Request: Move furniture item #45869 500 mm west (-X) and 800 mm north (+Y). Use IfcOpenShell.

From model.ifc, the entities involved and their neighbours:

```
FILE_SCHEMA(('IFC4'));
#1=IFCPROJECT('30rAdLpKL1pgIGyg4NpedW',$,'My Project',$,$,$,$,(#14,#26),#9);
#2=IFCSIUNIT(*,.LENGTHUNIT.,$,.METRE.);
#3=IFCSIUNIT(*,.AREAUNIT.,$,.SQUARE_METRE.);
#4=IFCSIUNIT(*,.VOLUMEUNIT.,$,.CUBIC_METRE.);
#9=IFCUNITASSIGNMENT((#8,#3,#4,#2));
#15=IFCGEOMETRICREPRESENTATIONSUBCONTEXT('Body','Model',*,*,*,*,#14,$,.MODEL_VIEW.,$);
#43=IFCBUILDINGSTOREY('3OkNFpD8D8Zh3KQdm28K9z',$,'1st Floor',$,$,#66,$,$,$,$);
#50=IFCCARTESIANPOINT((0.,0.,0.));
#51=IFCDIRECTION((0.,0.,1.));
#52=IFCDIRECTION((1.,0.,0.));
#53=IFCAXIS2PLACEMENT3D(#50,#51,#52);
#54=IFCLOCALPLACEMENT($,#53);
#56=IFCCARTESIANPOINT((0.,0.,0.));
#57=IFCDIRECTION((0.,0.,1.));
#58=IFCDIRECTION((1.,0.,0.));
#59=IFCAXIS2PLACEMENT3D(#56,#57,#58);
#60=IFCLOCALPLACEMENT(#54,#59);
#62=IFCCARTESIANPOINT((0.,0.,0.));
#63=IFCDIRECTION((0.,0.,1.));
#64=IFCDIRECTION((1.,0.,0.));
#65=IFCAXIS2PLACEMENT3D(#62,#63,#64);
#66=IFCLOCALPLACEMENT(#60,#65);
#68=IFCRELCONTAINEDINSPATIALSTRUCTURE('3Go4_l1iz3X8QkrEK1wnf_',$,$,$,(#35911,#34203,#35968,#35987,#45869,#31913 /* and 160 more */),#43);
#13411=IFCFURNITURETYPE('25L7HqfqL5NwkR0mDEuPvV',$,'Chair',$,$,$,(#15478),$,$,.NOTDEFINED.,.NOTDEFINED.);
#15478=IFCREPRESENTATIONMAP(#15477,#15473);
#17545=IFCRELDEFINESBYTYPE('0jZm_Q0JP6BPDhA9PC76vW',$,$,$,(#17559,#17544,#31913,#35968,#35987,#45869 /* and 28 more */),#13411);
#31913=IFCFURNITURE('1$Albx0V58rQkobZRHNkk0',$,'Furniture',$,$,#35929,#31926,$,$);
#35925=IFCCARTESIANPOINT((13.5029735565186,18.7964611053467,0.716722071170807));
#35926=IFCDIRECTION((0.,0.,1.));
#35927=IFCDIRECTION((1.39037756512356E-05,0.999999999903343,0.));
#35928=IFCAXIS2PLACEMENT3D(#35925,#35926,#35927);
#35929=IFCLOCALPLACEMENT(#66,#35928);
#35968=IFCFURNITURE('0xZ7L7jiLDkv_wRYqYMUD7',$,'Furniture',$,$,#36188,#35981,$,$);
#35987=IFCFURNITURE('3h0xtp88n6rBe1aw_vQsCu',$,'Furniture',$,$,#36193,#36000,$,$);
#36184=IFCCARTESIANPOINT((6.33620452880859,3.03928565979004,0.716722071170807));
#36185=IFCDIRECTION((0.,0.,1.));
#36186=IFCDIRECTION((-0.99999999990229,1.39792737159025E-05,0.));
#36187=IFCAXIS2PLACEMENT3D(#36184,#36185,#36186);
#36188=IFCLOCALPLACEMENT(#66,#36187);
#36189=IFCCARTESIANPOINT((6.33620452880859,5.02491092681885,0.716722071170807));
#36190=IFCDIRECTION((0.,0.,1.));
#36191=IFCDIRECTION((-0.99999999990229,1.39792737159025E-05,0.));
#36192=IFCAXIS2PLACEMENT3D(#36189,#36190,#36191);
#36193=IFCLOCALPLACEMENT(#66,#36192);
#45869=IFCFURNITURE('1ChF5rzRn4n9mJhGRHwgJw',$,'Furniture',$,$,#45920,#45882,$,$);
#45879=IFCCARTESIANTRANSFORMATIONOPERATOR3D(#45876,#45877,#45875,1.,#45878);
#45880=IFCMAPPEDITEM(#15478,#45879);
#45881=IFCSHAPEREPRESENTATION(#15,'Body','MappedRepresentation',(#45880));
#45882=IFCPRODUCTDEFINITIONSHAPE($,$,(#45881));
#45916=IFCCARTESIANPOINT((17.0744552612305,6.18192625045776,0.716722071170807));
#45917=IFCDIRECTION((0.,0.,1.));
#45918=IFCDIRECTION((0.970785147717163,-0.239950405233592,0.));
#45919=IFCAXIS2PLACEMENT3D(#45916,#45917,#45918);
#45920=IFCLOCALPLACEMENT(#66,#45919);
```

```python
import ifcopenshell
import ifcopenshell.api.geometry
import ifcopenshell.util.placement
import ifcopenshell.util.unit

model = ifcopenshell.open("model.ifc")
unit_scale = ifcopenshell.util.unit.calculate_unit_scale(model)

item = model.by_guid("1ChF5rzRn4n9mJhGRHwgJw")
matrix = ifcopenshell.util.placement.get_local_placement(item.ObjectPlacement)
matrix[0, 3] -= 0.5 / unit_scale
matrix[1, 3] += 0.8 / unit_scale
ifcopenshell.api.geometry.edit_object_placement(model, product=item, matrix=matrix, is_si=False)

print(ifcopenshell.util.placement.get_local_placement(item.ObjectPlacement).round(3) + 0.0)

model.write("model_edited.ifc")
```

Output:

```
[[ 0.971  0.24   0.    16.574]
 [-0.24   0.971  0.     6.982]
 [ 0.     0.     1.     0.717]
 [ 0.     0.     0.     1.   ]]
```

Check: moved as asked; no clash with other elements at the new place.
